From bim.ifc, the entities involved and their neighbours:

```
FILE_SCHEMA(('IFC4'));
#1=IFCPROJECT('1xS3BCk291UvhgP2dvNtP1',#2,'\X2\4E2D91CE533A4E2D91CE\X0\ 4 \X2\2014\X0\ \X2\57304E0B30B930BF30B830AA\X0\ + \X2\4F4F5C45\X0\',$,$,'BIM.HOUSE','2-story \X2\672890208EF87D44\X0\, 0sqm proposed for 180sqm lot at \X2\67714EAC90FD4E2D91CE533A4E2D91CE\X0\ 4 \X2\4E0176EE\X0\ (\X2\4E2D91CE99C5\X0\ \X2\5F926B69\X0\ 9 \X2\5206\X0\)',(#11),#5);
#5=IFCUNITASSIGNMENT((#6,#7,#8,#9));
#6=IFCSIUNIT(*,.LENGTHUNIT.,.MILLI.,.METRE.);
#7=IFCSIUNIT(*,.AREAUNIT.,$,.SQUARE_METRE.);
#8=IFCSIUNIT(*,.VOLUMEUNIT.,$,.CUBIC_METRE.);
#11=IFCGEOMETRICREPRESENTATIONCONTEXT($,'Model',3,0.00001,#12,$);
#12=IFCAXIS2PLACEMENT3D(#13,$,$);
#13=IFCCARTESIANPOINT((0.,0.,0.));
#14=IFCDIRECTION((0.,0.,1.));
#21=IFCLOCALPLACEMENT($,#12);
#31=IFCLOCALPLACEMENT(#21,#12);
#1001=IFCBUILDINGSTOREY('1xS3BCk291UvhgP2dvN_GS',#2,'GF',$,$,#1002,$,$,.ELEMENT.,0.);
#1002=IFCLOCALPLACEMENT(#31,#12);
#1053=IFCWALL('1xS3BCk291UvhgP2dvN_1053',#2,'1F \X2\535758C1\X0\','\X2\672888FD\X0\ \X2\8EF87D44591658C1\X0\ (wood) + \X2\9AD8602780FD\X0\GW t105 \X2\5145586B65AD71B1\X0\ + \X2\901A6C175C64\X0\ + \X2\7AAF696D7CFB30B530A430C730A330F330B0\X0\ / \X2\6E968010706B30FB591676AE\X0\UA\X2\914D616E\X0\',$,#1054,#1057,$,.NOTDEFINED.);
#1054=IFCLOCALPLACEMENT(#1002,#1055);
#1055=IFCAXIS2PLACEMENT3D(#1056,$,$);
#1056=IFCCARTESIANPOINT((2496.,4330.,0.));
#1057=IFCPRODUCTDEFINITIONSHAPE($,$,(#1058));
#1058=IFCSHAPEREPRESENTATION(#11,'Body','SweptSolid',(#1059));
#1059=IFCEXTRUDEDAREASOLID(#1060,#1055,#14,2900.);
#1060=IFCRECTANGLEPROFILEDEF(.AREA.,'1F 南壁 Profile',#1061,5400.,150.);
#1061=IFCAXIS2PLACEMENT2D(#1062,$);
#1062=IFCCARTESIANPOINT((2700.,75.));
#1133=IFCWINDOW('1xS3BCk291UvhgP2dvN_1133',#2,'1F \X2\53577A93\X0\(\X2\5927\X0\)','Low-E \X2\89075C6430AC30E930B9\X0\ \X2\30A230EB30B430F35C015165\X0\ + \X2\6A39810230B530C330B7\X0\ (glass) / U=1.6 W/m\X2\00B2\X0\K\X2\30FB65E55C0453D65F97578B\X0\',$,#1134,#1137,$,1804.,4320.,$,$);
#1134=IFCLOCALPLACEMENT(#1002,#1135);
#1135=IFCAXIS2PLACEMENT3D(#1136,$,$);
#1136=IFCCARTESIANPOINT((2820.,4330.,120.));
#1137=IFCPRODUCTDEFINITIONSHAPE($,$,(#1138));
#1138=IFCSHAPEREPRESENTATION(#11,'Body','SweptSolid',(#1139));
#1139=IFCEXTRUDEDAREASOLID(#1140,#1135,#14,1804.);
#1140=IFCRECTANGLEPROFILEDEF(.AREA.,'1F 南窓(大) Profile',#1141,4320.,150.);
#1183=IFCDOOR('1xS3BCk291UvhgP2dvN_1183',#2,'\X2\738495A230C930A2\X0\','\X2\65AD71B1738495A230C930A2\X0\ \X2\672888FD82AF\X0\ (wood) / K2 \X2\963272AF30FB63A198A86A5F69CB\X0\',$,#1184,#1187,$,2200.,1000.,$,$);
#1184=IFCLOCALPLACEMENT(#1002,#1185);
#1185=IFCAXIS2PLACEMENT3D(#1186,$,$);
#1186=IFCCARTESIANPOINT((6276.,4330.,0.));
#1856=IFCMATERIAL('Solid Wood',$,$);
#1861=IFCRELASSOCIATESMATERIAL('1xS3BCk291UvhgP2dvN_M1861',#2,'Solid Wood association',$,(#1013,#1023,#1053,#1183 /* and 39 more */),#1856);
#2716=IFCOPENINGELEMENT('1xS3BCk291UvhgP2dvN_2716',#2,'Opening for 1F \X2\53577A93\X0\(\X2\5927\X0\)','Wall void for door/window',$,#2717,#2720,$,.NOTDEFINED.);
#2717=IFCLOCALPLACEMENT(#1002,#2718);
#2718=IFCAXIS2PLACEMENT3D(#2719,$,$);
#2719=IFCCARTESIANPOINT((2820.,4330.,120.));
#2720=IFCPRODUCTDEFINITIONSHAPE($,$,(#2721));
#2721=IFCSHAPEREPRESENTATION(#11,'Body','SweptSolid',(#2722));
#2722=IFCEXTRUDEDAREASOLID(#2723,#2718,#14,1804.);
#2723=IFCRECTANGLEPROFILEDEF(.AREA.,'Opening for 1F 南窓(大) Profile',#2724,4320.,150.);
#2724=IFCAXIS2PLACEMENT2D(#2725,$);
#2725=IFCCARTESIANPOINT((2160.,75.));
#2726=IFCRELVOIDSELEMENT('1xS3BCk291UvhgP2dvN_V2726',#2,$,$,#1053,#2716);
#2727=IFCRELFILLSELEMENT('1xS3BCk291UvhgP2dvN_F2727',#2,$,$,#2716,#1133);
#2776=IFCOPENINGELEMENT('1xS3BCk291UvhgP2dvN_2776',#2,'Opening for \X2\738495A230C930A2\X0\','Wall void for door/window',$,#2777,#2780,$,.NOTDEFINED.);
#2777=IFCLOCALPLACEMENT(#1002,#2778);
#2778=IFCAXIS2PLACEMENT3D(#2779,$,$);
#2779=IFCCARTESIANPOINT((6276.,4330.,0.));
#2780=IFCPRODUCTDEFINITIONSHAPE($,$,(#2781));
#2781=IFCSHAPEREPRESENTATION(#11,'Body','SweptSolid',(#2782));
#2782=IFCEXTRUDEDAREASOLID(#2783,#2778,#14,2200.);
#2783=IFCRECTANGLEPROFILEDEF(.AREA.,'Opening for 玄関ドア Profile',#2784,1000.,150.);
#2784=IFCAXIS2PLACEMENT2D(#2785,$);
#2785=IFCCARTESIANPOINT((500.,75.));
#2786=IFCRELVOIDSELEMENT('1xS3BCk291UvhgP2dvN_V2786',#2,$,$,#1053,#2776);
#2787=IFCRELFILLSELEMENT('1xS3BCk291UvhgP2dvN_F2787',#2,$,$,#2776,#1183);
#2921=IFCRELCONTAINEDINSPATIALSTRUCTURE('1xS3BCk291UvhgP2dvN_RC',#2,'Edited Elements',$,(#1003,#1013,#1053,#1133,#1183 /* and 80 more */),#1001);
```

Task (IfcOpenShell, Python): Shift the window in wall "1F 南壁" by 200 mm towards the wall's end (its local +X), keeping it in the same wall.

```python
import ifcopenshell
import ifcopenshell.api.geometry
import ifcopenshell.util.placement
import ifcopenshell.util.unit

model = ifcopenshell.open("bim.ifc")
unit_scale = ifcopenshell.util.unit.calculate_unit_scale(model)

window = model.by_id(1133)
opening = window.FillsVoids[0].RelatingOpeningElement
wall = opening.VoidsElements[0].RelatingBuildingElement

wall_matrix = ifcopenshell.util.placement.get_local_placement(wall.ObjectPlacement)
shift = wall_matrix[:3, 0] * 0.2 / unit_scale
before = ifcopenshell.util.placement.get_local_placement(window.ObjectPlacement)[:3, 3].copy()

# The window is not placed relative to its opening, so move both.
for product in (opening, window):
    matrix = ifcopenshell.util.placement.get_local_placement(product.ObjectPlacement)
    matrix[:3, 3] += shift
    ifcopenshell.api.geometry.edit_object_placement(model, product=product, matrix=matrix, is_si=False)

after = ifcopenshell.util.placement.get_local_placement(window.ObjectPlacement)[:3, 3]
print("window moved by", (after - before).round(3) + 0.0)

model.write("bim_v2.ifc")
```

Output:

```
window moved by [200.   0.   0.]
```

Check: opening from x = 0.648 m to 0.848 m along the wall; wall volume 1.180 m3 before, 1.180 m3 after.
